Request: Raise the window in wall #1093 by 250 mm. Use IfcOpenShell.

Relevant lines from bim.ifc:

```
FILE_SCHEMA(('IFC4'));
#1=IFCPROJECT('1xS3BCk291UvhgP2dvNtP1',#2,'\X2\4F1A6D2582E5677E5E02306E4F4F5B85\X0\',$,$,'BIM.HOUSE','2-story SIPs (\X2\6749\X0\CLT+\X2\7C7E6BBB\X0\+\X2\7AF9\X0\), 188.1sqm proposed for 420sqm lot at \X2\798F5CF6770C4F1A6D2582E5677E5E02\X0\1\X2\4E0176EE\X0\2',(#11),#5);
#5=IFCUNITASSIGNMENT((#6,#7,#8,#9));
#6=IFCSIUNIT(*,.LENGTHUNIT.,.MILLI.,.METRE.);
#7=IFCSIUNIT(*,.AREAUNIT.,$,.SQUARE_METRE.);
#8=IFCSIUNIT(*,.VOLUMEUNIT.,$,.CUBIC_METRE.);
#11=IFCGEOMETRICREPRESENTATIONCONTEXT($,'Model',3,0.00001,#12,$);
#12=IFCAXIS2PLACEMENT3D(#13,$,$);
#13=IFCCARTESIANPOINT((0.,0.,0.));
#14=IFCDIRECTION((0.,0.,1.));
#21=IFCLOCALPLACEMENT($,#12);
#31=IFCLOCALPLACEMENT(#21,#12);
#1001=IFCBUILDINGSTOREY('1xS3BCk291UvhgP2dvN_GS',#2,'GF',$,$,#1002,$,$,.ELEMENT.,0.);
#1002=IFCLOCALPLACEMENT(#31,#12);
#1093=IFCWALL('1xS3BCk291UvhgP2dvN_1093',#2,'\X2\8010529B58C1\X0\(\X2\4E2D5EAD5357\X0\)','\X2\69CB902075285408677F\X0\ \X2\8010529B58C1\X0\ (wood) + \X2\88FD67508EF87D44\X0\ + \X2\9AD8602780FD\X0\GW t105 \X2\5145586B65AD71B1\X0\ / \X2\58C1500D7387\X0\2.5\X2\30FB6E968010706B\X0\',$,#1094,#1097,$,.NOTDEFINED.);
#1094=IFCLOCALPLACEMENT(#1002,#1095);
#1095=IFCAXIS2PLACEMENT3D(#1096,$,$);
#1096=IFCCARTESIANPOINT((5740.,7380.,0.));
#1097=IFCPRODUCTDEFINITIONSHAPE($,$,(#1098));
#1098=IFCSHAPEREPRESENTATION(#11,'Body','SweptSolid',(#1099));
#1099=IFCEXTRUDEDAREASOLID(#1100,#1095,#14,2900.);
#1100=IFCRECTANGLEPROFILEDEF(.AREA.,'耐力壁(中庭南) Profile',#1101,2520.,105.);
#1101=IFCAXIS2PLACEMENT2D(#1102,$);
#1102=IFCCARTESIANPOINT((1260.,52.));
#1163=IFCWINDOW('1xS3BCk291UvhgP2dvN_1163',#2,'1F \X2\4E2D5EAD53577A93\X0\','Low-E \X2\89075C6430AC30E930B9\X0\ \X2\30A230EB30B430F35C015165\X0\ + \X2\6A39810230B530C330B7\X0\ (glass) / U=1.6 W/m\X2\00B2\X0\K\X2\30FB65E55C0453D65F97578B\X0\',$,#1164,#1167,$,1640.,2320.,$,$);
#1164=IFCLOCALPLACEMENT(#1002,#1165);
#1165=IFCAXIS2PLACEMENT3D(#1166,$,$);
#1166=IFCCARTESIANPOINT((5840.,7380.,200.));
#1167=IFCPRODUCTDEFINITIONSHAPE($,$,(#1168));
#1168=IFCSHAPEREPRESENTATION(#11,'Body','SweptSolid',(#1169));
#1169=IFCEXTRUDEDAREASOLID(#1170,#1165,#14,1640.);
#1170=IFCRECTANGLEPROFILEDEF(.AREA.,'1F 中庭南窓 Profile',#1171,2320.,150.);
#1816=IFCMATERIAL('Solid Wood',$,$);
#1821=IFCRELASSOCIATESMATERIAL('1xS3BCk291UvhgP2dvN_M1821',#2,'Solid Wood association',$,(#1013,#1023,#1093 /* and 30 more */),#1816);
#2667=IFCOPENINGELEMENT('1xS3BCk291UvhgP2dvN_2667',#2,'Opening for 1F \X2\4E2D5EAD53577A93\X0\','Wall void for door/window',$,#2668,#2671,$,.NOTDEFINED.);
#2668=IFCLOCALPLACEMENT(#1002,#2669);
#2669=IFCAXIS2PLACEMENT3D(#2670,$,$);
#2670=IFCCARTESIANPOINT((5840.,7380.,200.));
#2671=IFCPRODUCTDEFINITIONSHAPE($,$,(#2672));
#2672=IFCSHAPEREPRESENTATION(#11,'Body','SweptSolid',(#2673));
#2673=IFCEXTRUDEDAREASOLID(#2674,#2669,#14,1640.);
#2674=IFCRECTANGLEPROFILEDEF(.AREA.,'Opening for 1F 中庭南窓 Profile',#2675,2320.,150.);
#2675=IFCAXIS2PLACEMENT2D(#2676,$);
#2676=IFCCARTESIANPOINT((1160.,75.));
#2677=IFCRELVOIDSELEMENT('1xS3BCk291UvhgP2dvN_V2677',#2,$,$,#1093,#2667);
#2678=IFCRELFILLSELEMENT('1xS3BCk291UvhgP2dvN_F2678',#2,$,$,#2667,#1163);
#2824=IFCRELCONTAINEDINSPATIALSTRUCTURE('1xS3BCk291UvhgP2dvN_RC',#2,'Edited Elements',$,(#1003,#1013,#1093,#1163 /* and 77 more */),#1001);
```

```python
import numpy as np
import ifcopenshell
import ifcopenshell.api.geometry
import ifcopenshell.util.placement
import ifcopenshell.util.unit

model = ifcopenshell.open("bim.ifc")
unit_scale = ifcopenshell.util.unit.calculate_unit_scale(model)

window = model.by_guid("1xS3BCk291UvhgP2dvN_1163")
opening = window.FillsVoids[0].RelatingOpeningElement
dz = 0.25 / unit_scale

shift = np.array([0.0, 0.0, dz])
# The window is not placed relative to its opening, so move both.
for product in (opening, window):
    matrix = ifcopenshell.util.placement.get_local_placement(product.ObjectPlacement)
    matrix[:3, 3] += shift
    ifcopenshell.api.geometry.edit_object_placement(model, product=product, matrix=matrix, is_si=False)

print(f"moved by {dz * unit_scale:+.3f} m")

model.write("bim_v2.ifc")
```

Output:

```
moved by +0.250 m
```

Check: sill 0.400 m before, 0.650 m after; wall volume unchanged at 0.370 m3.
